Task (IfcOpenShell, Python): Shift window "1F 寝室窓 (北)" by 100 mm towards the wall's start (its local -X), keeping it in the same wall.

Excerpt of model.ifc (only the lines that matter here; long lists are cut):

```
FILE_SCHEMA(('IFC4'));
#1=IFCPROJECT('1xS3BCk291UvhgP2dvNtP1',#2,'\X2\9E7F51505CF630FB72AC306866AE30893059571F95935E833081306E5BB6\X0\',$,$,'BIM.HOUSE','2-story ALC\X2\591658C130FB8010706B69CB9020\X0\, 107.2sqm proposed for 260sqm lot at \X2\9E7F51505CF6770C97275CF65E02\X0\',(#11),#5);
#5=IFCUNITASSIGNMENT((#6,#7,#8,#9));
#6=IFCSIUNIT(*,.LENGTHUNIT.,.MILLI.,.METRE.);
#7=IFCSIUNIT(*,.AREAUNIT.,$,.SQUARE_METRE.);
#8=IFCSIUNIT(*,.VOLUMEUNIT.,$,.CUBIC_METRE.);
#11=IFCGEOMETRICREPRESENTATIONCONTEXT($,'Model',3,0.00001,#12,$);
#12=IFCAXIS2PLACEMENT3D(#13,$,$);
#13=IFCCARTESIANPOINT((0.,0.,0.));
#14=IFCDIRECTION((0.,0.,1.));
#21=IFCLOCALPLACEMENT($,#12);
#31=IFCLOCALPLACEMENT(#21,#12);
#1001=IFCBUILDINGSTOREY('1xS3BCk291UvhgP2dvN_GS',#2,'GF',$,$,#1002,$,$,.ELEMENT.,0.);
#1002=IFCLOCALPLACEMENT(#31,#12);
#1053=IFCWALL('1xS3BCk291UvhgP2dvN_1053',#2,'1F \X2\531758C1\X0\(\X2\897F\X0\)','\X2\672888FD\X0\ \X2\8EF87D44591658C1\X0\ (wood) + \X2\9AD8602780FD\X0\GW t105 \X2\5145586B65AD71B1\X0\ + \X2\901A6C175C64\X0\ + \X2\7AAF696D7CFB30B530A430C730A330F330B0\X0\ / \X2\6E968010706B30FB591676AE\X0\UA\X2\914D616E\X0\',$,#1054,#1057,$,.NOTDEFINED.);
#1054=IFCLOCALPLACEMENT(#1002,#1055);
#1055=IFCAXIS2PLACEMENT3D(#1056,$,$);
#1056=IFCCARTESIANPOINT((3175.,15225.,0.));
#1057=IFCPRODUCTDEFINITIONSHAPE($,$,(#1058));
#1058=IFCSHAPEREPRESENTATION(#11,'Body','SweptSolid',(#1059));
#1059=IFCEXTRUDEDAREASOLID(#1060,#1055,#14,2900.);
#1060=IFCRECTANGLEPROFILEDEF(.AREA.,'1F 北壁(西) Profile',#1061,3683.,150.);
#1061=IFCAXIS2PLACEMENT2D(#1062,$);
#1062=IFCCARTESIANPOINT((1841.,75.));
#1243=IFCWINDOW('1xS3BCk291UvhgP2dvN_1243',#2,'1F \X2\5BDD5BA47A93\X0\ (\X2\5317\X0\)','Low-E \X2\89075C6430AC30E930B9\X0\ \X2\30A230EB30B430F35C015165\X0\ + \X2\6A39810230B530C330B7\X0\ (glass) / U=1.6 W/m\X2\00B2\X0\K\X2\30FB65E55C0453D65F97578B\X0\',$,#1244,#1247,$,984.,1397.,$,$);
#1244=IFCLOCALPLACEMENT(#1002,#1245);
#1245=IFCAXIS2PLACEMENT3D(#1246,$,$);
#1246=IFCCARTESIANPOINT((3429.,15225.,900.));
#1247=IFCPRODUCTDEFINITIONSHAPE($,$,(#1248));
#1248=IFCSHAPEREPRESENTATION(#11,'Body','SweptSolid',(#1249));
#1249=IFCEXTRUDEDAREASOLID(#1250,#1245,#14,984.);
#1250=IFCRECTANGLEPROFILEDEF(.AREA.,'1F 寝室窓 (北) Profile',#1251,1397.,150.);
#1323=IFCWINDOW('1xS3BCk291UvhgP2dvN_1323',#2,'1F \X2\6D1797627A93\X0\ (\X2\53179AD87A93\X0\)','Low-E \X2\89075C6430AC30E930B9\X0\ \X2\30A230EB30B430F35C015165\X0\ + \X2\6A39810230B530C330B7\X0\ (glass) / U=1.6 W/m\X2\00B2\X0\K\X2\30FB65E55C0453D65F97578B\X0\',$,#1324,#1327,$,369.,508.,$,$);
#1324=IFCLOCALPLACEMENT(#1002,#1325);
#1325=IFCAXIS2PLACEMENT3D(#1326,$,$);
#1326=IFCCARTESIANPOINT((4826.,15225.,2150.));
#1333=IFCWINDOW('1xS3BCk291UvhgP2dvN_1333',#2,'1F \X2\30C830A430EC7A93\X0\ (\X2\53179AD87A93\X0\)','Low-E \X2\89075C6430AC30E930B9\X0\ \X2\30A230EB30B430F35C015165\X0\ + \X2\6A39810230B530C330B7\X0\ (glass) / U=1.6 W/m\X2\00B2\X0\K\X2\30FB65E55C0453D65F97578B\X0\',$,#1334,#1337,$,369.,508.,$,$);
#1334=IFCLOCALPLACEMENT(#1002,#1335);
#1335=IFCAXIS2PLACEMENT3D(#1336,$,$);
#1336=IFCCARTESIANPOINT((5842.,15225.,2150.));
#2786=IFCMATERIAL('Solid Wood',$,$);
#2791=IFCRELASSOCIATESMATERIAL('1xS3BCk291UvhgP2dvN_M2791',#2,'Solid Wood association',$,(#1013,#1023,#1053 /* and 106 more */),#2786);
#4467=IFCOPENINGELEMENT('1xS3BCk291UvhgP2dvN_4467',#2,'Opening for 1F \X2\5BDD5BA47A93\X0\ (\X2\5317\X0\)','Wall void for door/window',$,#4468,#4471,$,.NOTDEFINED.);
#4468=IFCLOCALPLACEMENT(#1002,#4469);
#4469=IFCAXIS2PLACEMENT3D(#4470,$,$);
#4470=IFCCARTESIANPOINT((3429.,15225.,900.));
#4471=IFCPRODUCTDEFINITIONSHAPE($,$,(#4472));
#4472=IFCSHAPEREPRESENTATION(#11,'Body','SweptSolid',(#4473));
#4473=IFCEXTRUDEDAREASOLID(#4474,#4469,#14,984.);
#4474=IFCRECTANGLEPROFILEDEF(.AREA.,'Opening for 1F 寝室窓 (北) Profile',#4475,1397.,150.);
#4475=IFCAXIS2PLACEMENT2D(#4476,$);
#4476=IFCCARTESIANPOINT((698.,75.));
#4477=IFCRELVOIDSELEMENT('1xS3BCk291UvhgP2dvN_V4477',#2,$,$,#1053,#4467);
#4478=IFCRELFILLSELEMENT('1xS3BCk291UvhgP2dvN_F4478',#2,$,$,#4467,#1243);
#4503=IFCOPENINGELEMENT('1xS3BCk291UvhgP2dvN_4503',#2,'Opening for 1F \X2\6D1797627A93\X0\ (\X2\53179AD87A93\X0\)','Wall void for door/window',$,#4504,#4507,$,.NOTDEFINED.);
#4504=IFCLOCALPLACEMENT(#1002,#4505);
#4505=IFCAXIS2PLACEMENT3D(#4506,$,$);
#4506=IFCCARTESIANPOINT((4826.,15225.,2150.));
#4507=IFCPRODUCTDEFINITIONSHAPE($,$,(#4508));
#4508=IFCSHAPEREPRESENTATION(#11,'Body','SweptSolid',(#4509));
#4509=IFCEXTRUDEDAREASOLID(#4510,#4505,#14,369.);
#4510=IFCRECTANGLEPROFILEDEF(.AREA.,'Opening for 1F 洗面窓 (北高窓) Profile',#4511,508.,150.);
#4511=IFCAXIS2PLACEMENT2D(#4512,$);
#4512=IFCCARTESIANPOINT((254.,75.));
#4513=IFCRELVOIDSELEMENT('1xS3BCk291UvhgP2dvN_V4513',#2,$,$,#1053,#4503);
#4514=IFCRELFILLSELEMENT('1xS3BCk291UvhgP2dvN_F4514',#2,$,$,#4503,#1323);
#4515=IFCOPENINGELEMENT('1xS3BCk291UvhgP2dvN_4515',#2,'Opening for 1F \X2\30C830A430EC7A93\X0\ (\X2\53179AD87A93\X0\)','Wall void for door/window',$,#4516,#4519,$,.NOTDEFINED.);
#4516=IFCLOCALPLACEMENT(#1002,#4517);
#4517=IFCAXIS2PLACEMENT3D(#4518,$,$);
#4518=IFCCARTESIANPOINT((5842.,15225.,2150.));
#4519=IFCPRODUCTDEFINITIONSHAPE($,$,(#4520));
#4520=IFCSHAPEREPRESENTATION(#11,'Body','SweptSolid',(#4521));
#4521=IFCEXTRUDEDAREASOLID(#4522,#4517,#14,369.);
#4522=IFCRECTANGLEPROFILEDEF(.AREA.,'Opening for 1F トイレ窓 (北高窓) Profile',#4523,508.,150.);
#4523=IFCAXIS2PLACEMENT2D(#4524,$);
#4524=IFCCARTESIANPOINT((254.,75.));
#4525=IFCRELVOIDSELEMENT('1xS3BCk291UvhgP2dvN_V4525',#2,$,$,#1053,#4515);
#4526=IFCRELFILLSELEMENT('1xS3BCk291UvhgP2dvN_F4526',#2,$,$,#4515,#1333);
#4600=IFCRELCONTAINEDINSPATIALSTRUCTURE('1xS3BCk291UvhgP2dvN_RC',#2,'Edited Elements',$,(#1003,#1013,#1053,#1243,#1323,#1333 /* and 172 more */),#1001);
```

```python
import ifcopenshell
import ifcopenshell.api.geometry
import ifcopenshell.util.placement
import ifcopenshell.util.unit

model = ifcopenshell.open("model.ifc")
unit_scale = ifcopenshell.util.unit.calculate_unit_scale(model)

window = model.by_id(1243)
opening = window.FillsVoids[0].RelatingOpeningElement
wall = opening.VoidsElements[0].RelatingBuildingElement

wall_matrix = ifcopenshell.util.placement.get_local_placement(wall.ObjectPlacement)
shift = wall_matrix[:3, 0] * -0.1 / unit_scale
before = ifcopenshell.util.placement.get_local_placement(window.ObjectPlacement)[:3, 3].copy()

# The window is not placed relative to its opening, so move both.
for product in (opening, window):
    matrix = ifcopenshell.util.placement.get_local_placement(product.ObjectPlacement)
    matrix[:3, 3] += shift
    ifcopenshell.api.geometry.edit_object_placement(model, product=product, matrix=matrix, is_si=False)

after = ifcopenshell.util.placement.get_local_placement(window.ObjectPlacement)[:3, 3]
print("window moved by", (after - before).round(3) + 0.0)

model.write("model-out.ifc")
```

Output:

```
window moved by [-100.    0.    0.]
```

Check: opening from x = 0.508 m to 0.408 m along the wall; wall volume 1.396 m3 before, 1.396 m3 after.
